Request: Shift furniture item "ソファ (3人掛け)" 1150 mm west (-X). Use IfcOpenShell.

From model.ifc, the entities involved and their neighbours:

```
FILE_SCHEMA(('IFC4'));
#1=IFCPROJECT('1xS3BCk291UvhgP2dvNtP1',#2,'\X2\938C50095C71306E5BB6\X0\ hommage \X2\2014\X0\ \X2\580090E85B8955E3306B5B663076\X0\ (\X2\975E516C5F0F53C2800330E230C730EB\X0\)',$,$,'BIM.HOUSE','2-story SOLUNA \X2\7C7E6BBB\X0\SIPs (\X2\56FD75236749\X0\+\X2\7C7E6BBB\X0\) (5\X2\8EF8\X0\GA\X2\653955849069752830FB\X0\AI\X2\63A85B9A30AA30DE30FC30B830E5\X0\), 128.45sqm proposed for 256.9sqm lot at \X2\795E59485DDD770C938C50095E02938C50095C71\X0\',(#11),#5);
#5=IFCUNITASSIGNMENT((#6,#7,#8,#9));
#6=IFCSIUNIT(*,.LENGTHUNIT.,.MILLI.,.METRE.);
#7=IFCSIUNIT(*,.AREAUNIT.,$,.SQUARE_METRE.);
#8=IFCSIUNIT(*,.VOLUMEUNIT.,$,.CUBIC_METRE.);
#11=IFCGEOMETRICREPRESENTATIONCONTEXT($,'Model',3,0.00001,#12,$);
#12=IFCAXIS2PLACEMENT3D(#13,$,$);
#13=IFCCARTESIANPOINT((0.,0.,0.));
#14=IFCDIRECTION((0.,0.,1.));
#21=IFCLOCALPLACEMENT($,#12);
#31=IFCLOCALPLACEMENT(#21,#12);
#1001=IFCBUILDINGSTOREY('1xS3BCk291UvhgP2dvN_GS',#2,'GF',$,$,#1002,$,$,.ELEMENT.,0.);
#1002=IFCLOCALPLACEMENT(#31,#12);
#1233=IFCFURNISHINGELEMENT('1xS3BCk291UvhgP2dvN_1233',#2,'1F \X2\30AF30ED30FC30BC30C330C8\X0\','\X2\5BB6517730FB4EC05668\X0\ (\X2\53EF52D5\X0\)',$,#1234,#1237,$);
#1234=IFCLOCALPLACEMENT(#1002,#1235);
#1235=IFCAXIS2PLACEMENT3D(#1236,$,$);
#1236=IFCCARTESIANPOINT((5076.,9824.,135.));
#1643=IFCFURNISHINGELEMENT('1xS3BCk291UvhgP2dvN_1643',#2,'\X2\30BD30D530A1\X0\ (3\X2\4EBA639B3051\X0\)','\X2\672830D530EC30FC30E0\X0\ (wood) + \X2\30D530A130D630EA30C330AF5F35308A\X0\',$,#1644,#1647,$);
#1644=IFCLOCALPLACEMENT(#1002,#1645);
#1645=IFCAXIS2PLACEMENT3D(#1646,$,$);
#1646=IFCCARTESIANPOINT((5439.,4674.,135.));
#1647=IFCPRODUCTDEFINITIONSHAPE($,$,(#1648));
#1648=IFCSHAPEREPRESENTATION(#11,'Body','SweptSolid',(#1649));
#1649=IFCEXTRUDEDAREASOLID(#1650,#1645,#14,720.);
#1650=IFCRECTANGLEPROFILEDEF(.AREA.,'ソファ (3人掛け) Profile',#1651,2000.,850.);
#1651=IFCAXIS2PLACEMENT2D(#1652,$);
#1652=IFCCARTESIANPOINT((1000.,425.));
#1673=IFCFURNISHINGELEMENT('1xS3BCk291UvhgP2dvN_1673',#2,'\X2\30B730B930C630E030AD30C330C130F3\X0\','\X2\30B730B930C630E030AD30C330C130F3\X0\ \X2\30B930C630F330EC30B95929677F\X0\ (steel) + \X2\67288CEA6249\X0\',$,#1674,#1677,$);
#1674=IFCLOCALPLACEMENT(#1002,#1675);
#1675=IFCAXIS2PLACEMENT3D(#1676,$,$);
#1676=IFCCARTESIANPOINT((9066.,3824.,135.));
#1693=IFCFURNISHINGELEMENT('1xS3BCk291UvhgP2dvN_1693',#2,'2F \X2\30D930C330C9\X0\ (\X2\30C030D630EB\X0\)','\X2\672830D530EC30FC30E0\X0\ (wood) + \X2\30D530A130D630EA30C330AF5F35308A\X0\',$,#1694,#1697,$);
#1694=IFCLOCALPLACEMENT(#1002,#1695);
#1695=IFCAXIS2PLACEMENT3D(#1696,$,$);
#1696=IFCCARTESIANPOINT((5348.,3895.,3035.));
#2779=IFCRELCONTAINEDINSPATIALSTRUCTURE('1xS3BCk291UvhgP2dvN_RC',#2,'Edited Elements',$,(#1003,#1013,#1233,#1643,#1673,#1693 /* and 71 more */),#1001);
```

```python
import ifcopenshell
import ifcopenshell.api.geometry
import ifcopenshell.util.placement
import ifcopenshell.util.unit

model = ifcopenshell.open("model.ifc")
unit_scale = ifcopenshell.util.unit.calculate_unit_scale(model)

item = model.by_guid("1xS3BCk291UvhgP2dvN_1643")
matrix = ifcopenshell.util.placement.get_local_placement(item.ObjectPlacement)
matrix[0, 3] -= 1.15 / unit_scale
ifcopenshell.api.geometry.edit_object_placement(model, product=item, matrix=matrix, is_si=False)

print(ifcopenshell.util.placement.get_local_placement(item.ObjectPlacement).round(3) + 0.0)

model.write("model_v2.ifc")
```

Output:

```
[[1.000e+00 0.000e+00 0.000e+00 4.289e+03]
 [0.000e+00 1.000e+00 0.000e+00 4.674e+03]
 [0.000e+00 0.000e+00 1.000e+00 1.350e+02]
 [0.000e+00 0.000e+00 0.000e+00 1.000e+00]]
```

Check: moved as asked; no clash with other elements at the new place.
